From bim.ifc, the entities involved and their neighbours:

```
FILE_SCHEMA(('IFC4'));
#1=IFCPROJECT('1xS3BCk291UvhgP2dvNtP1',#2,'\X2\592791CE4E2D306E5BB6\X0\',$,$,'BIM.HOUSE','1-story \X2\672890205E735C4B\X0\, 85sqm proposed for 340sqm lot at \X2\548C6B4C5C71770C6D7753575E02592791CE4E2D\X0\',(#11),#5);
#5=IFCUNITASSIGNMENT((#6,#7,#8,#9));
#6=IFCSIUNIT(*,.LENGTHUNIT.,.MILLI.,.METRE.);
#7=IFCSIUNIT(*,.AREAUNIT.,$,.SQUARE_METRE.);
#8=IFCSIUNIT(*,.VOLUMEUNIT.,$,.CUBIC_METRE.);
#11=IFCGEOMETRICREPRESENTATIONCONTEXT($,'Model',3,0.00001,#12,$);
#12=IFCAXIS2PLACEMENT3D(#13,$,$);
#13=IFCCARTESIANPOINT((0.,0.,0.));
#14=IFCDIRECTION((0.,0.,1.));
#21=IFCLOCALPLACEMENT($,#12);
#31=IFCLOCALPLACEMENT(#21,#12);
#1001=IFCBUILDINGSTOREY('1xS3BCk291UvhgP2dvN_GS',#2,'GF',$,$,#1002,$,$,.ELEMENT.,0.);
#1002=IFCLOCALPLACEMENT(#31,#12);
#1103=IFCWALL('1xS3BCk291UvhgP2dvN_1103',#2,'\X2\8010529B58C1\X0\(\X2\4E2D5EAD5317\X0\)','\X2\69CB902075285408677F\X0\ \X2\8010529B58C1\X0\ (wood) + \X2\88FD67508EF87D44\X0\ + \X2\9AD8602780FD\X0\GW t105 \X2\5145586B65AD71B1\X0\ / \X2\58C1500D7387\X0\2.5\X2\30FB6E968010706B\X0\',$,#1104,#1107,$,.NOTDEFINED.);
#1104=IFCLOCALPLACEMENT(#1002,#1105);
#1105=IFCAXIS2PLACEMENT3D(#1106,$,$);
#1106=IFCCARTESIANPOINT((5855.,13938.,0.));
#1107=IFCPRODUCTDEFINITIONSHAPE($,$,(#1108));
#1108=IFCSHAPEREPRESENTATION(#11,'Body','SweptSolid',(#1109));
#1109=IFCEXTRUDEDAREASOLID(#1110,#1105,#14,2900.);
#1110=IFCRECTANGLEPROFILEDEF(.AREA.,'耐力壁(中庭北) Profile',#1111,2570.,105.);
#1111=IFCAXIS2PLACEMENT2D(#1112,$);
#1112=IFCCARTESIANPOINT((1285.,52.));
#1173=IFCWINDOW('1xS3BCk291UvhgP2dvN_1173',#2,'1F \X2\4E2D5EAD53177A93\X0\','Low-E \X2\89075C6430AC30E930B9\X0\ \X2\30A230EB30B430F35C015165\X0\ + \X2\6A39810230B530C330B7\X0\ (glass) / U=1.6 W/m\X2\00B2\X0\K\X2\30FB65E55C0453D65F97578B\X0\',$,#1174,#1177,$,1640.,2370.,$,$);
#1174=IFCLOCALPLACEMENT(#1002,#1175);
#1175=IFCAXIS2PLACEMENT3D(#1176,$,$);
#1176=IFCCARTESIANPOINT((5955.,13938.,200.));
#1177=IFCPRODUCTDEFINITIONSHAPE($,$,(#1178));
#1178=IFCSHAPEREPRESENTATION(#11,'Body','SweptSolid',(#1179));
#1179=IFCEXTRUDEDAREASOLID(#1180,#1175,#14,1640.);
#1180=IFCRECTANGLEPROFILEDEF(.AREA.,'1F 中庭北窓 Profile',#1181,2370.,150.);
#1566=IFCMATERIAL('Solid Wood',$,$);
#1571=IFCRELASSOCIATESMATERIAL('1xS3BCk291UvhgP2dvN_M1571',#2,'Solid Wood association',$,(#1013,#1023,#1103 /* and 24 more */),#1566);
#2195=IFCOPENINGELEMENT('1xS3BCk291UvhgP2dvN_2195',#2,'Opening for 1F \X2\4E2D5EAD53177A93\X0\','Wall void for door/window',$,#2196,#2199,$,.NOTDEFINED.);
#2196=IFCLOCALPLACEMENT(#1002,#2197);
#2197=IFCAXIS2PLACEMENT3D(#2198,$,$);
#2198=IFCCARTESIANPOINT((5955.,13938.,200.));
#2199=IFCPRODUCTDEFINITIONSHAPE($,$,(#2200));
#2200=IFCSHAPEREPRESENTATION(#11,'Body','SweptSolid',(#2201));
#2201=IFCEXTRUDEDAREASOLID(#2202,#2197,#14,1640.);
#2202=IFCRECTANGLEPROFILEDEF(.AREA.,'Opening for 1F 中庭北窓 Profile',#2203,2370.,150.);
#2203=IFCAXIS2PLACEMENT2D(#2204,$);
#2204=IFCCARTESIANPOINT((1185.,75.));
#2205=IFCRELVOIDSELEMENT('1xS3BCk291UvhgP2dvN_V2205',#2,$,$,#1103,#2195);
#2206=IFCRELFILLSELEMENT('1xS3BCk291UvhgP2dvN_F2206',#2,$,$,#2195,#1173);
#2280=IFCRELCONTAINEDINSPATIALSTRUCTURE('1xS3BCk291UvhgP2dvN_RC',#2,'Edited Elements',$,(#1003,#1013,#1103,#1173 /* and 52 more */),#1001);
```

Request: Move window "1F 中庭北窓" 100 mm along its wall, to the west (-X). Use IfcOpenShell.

```python
import ifcopenshell
import ifcopenshell.api.geometry
import ifcopenshell.util.placement

model = ifcopenshell.open("bim.ifc")

window = model.by_guid("1xS3BCk291UvhgP2dvN_1173")
opening = window.FillsVoids[0].RelatingOpeningElement
wall = opening.VoidsElements[0].RelatingBuildingElement

wall_matrix = ifcopenshell.util.placement.get_local_placement(wall.ObjectPlacement)
shift = wall_matrix[:3, 0] * -100.0
before = ifcopenshell.util.placement.get_local_placement(window.ObjectPlacement)[:3, 3].copy()

# The window is not placed relative to its opening, so move both.
for product in (opening, window):
    matrix = ifcopenshell.util.placement.get_local_placement(product.ObjectPlacement)
    matrix[:3, 3] += shift
    ifcopenshell.api.geometry.edit_object_placement(model, product=product, matrix=matrix, is_si=False)

after = ifcopenshell.util.placement.get_local_placement(window.ObjectPlacement)[:3, 3]
print("window moved by", (after - before).round(3) + 0.0)

model.write("bim-out.ifc")
```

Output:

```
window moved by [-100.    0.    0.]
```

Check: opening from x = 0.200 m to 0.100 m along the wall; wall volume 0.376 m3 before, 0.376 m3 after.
